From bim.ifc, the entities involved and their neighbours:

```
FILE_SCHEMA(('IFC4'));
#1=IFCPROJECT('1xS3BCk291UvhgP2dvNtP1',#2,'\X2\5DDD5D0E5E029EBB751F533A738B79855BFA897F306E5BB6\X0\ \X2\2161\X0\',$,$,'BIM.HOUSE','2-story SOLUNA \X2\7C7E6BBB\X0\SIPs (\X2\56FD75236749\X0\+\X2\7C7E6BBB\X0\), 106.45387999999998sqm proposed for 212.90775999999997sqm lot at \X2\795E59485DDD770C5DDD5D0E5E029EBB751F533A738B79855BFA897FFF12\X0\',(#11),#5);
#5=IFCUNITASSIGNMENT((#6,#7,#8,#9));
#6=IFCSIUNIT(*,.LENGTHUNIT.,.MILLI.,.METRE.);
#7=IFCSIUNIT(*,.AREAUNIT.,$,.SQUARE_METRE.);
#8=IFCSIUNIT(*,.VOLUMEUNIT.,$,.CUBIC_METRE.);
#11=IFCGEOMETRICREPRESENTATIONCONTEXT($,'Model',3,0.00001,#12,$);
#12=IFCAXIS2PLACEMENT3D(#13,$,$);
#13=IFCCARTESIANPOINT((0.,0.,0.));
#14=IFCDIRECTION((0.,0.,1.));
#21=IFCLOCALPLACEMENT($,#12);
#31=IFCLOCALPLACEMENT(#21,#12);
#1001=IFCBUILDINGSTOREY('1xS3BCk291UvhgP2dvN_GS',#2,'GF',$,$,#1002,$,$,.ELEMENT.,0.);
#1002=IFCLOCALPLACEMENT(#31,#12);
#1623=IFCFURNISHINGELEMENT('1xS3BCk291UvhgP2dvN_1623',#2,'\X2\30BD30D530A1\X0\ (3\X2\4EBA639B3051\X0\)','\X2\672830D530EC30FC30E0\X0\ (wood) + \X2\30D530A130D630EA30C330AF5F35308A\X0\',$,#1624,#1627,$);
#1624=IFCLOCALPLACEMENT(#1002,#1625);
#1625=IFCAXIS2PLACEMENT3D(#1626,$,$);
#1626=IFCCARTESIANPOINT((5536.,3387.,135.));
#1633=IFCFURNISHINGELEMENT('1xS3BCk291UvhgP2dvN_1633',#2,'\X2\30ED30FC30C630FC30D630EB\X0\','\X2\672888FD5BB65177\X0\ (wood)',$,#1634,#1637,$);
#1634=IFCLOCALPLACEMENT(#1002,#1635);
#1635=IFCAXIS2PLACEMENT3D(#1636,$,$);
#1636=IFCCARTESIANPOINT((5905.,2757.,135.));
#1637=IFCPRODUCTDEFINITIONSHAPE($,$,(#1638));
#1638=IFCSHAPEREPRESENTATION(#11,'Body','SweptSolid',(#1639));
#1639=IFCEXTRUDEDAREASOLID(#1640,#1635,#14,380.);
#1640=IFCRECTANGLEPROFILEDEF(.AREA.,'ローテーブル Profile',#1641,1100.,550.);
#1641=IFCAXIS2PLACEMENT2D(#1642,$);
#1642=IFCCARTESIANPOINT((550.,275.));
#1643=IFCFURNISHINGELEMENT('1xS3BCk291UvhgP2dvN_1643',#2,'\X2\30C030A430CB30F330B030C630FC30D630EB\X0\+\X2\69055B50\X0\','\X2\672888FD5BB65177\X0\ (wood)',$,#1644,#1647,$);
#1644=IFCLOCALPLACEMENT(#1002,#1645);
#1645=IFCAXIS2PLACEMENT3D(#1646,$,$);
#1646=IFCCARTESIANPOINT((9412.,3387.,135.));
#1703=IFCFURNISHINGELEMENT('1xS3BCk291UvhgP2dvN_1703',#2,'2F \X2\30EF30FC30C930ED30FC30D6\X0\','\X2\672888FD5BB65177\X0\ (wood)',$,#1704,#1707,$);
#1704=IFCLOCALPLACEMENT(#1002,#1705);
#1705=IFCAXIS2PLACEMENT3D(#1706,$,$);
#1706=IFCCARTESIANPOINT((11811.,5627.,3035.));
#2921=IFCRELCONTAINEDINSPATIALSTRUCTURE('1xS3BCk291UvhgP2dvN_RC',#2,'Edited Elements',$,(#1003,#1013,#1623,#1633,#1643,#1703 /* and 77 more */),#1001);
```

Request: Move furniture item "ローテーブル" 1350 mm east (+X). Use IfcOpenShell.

```python
import ifcopenshell
import ifcopenshell.api.geometry
import ifcopenshell.util.placement

model = ifcopenshell.open("bim.ifc")

item = model.by_id(1633)
matrix = ifcopenshell.util.placement.get_local_placement(item.ObjectPlacement)
matrix[0, 3] += 1350.0
ifcopenshell.api.geometry.edit_object_placement(model, product=item, matrix=matrix, is_si=False)

print(ifcopenshell.util.placement.get_local_placement(item.ObjectPlacement).round(3) + 0.0)

model.write("bim_rev.ifc")
```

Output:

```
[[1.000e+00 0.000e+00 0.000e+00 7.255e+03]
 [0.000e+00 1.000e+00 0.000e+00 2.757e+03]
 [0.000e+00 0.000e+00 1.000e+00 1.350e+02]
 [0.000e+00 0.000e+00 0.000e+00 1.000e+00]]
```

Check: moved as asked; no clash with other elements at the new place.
